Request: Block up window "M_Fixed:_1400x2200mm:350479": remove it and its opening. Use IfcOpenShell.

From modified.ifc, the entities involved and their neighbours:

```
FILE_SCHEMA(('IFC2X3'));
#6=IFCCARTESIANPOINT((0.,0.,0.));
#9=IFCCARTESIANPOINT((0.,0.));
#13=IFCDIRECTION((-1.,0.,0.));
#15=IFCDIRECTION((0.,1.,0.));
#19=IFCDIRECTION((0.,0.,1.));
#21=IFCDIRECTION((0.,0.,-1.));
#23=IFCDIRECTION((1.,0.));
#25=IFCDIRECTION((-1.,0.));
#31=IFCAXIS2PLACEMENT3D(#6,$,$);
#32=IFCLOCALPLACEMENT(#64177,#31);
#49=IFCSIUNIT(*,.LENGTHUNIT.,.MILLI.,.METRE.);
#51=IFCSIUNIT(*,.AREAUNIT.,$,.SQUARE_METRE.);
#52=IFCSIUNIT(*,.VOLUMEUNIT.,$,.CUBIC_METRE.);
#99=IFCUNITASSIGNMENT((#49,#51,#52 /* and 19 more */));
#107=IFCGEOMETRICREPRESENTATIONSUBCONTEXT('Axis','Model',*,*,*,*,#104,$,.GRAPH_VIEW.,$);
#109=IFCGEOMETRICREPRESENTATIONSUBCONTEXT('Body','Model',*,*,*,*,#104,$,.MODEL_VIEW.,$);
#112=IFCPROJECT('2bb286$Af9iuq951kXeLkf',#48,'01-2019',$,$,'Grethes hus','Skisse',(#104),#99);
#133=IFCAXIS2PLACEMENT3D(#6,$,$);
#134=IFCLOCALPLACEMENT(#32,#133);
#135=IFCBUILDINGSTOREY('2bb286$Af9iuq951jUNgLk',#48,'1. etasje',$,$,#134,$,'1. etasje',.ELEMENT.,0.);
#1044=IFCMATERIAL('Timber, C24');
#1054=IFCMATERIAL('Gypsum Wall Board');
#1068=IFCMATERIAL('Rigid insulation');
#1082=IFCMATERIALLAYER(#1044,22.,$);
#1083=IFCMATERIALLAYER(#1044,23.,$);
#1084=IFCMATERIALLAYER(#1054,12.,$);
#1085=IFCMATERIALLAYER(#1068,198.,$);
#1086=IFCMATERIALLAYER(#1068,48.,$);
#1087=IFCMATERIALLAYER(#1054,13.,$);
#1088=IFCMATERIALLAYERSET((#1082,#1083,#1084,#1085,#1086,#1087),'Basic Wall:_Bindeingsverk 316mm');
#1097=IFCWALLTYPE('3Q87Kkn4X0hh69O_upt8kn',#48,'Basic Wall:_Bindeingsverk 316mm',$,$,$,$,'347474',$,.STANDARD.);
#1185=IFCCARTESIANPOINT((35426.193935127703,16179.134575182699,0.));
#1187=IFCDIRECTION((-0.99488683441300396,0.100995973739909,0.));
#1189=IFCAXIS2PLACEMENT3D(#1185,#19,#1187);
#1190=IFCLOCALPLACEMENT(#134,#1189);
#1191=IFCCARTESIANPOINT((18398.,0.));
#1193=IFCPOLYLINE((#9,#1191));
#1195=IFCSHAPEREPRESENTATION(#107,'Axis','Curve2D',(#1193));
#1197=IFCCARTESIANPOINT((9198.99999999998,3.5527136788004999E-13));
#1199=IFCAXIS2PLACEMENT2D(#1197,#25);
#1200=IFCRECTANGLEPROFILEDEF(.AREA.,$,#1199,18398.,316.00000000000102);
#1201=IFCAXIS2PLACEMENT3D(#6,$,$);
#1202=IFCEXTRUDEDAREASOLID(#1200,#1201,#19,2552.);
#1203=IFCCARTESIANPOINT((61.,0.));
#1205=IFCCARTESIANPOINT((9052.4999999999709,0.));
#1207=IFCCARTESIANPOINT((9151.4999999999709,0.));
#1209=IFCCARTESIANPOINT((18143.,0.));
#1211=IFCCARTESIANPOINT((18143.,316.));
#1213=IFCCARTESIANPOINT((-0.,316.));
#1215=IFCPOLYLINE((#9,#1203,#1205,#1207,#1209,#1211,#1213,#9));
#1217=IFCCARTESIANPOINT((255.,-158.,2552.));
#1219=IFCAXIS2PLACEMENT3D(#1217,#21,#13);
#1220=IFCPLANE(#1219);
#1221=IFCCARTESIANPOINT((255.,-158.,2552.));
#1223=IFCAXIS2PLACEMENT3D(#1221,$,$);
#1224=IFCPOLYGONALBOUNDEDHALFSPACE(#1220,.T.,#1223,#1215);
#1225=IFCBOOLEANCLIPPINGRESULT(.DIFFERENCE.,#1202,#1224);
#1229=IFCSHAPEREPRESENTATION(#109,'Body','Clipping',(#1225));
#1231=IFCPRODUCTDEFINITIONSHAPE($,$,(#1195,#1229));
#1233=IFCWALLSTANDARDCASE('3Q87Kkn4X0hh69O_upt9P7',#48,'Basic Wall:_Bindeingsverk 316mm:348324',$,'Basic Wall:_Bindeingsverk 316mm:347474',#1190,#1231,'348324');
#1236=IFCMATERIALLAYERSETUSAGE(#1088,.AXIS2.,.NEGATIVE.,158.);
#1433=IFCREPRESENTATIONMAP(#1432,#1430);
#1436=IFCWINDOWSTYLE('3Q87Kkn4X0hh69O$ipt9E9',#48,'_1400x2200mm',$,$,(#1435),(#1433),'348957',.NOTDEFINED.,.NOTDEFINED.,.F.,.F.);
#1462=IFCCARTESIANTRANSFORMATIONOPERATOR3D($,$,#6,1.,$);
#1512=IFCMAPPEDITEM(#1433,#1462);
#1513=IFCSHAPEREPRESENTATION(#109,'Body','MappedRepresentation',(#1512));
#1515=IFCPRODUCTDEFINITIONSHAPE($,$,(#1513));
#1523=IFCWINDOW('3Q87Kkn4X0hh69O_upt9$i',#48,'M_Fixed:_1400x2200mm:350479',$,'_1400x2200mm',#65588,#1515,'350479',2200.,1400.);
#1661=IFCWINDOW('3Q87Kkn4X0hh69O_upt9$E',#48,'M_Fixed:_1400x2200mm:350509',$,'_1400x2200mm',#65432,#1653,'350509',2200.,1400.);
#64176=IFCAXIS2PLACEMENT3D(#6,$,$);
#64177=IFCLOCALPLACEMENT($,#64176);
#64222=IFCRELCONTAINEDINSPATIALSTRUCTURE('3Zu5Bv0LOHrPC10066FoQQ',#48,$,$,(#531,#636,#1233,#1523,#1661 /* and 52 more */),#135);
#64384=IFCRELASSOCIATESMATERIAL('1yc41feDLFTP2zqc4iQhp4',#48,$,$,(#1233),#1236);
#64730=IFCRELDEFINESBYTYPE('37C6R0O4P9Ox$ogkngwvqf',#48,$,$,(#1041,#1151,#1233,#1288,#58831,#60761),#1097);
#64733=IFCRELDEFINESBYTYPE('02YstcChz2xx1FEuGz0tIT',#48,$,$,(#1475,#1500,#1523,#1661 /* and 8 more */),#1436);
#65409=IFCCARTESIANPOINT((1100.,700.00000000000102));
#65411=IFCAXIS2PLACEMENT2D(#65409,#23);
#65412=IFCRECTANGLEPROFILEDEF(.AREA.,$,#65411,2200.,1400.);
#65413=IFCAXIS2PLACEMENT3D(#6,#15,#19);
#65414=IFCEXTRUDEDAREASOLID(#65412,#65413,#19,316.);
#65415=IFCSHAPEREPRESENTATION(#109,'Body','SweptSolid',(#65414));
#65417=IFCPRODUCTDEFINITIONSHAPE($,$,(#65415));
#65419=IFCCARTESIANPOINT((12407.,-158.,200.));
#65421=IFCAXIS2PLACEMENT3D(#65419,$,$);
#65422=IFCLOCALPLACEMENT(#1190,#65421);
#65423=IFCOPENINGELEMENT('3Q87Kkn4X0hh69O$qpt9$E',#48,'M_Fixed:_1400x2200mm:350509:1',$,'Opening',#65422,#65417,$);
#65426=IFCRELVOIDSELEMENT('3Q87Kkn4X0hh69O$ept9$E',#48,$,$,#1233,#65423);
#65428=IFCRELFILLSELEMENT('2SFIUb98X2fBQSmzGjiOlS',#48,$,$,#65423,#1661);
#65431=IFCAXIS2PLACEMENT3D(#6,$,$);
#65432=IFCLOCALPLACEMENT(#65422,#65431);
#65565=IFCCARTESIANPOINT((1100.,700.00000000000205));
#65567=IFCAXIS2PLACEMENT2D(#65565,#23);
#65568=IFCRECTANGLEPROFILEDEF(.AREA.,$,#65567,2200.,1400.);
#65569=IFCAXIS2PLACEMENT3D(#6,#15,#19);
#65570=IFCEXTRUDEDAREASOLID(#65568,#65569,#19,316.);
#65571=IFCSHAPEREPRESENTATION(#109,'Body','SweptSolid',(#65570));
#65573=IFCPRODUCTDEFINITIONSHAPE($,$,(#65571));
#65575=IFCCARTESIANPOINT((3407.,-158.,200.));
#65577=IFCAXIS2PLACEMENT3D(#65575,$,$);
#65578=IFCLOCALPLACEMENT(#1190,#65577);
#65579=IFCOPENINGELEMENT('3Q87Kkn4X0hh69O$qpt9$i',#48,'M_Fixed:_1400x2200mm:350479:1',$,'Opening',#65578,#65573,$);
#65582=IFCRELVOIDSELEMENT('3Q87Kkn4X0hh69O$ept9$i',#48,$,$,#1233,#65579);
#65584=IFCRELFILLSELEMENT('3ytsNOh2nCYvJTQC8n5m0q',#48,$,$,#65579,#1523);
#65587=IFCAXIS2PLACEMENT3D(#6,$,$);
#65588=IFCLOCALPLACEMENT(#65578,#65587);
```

```python
import ifcopenshell
import ifcopenshell.api.feature
import ifcopenshell.api.root
import ifcopenshell.geom
import ifcopenshell.util.shape

model = ifcopenshell.open("modified.ifc")
settings = ifcopenshell.geom.settings()


def volume(element):
    """Net volume in cubic metres, openings subtracted."""
    shape = ifcopenshell.geom.create_shape(settings, element)
    return ifcopenshell.util.shape.get_volume(shape.geometry)


window = model.by_id(1523)
opening = window.FillsVoids[0].RelatingOpeningElement
wall = opening.VoidsElements[0].RelatingBuildingElement
before = volume(wall)

ifcopenshell.api.root.remove_product(model, product=window)
ifcopenshell.api.feature.remove_feature(model, feature=opening)

after = volume(wall)

print(f"wall volume {before:.3f} -> {after:.3f} m3")

model.write("modified-out.ifc")
```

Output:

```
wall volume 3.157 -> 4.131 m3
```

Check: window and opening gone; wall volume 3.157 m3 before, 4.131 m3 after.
